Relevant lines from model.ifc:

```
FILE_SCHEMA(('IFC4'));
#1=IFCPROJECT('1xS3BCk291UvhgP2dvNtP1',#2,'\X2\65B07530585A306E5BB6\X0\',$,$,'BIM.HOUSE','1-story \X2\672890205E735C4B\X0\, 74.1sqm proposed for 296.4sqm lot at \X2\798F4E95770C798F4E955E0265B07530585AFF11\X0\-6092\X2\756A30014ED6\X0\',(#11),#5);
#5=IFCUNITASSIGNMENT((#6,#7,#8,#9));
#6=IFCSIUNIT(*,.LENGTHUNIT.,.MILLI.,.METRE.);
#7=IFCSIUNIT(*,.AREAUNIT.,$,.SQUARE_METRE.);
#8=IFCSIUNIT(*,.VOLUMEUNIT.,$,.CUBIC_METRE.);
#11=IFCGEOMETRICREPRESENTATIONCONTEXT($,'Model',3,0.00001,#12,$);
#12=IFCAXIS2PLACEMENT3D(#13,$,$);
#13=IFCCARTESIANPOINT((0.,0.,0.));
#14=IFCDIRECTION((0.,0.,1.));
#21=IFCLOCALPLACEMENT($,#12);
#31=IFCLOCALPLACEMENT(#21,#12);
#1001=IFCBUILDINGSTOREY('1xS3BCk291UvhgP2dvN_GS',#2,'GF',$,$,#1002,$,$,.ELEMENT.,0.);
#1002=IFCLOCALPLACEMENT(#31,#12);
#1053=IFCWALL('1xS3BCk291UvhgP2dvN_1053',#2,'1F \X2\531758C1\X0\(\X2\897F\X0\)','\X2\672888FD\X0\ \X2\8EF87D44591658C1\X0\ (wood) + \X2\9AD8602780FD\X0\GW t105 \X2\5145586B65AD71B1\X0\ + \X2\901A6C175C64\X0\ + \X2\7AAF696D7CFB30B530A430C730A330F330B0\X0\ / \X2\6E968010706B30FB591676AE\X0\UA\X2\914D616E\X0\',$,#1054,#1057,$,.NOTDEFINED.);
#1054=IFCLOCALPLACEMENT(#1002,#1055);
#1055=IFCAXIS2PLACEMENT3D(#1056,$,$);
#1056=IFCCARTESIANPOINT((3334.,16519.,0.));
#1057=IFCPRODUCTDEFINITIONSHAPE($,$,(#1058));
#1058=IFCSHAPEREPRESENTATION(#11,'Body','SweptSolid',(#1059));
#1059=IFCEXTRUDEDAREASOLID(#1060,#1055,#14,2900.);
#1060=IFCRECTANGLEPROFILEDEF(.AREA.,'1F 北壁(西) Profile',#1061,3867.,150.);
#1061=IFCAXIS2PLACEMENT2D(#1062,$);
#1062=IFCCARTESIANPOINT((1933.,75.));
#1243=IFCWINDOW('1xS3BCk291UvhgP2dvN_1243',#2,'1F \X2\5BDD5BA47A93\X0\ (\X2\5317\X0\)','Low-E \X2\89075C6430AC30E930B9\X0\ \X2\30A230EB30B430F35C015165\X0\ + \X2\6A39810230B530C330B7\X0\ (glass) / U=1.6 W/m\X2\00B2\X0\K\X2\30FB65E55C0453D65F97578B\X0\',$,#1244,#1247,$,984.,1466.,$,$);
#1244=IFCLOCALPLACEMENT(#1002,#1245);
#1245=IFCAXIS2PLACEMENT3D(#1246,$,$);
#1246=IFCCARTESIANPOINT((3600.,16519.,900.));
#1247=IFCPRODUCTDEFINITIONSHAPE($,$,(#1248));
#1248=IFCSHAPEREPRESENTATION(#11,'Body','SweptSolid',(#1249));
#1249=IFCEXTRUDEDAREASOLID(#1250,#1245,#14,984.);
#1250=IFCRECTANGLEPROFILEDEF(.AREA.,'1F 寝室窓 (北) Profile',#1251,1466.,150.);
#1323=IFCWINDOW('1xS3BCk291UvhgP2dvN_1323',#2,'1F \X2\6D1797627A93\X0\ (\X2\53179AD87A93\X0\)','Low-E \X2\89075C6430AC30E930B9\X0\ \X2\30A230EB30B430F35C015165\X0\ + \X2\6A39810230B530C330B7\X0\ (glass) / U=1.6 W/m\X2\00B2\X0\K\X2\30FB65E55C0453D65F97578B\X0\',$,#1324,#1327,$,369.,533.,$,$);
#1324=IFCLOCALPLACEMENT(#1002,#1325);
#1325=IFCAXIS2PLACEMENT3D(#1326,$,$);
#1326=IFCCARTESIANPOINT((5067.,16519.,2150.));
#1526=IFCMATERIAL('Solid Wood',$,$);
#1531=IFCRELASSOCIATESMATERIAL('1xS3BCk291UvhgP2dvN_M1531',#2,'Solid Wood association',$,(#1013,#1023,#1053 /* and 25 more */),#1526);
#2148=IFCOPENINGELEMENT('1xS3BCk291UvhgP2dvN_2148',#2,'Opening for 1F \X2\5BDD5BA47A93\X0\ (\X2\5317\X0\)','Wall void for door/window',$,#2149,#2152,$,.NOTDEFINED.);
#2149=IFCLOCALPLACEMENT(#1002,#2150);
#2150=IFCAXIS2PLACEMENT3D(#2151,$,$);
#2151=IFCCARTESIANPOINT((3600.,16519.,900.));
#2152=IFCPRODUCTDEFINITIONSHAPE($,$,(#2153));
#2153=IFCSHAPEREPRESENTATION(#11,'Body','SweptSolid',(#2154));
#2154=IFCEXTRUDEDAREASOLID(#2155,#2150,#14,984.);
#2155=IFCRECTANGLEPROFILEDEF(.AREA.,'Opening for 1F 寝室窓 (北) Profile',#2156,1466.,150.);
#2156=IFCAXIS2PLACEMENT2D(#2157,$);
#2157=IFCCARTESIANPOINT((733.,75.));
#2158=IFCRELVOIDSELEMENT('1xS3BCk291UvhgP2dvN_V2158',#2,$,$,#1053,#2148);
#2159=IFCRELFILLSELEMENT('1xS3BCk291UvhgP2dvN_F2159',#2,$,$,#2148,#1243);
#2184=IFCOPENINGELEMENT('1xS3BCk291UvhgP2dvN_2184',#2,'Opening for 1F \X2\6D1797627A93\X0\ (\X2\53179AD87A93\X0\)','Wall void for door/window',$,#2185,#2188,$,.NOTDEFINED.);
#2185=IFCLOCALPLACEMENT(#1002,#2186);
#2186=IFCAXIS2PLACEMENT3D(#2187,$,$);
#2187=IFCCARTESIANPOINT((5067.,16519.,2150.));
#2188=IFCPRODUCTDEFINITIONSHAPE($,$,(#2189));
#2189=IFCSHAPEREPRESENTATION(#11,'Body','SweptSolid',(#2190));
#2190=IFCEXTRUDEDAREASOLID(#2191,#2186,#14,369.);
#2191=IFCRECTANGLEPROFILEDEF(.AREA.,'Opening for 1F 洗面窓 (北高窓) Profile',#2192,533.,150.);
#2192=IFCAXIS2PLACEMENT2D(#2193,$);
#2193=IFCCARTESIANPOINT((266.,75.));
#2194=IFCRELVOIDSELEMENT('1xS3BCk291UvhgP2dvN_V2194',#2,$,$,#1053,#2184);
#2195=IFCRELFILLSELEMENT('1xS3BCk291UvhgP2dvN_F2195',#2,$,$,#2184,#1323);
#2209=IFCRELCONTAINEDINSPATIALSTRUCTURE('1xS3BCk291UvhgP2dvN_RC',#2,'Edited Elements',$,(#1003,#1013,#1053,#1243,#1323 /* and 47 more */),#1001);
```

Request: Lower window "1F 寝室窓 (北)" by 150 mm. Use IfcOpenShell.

```python
import numpy as np
import ifcopenshell
import ifcopenshell.api.geometry
import ifcopenshell.util.placement
import ifcopenshell.util.unit

model = ifcopenshell.open("model.ifc")
unit_scale = ifcopenshell.util.unit.calculate_unit_scale(model)

window = model.by_guid("1xS3BCk291UvhgP2dvN_1243")
opening = window.FillsVoids[0].RelatingOpeningElement
dz = -0.15 / unit_scale

shift = np.array([0.0, 0.0, dz])
# The window is not placed relative to its opening, so move both.
for product in (opening, window):
    matrix = ifcopenshell.util.placement.get_local_placement(product.ObjectPlacement)
    matrix[:3, 3] += shift
    ifcopenshell.api.geometry.edit_object_placement(model, product=product, matrix=matrix, is_si=False)

print(f"moved by {dz * unit_scale:+.3f} m")

model.write("model_edited.ifc")
```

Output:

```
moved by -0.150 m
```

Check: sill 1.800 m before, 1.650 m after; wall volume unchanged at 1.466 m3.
